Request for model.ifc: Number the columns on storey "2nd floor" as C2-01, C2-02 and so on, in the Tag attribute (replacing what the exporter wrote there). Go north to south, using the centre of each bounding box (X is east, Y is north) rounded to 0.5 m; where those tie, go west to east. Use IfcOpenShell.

First a look at what the model holds.

```python
import ifcopenshell
import ifcopenshell.util.element
import ifcopenshell.util.placement

model = ifcopenshell.open("model.ifc")
print(model.schema)
storey = next(s for s in model.by_type("IfcBuildingStorey") if s.Name == "2nd floor")
columns = [e for e in ifcopenshell.util.element.get_decomposition(storey) if e.is_a("IfcColumn")]
for e in sorted(columns, key=lambda e: e.id()):
    origin = ifcopenshell.util.placement.get_local_placement(e.ObjectPlacement)[:3, 3]
    print(e.id(), e.Tag, e.Name, origin.round(2) + 0.0, sep=" | ")
```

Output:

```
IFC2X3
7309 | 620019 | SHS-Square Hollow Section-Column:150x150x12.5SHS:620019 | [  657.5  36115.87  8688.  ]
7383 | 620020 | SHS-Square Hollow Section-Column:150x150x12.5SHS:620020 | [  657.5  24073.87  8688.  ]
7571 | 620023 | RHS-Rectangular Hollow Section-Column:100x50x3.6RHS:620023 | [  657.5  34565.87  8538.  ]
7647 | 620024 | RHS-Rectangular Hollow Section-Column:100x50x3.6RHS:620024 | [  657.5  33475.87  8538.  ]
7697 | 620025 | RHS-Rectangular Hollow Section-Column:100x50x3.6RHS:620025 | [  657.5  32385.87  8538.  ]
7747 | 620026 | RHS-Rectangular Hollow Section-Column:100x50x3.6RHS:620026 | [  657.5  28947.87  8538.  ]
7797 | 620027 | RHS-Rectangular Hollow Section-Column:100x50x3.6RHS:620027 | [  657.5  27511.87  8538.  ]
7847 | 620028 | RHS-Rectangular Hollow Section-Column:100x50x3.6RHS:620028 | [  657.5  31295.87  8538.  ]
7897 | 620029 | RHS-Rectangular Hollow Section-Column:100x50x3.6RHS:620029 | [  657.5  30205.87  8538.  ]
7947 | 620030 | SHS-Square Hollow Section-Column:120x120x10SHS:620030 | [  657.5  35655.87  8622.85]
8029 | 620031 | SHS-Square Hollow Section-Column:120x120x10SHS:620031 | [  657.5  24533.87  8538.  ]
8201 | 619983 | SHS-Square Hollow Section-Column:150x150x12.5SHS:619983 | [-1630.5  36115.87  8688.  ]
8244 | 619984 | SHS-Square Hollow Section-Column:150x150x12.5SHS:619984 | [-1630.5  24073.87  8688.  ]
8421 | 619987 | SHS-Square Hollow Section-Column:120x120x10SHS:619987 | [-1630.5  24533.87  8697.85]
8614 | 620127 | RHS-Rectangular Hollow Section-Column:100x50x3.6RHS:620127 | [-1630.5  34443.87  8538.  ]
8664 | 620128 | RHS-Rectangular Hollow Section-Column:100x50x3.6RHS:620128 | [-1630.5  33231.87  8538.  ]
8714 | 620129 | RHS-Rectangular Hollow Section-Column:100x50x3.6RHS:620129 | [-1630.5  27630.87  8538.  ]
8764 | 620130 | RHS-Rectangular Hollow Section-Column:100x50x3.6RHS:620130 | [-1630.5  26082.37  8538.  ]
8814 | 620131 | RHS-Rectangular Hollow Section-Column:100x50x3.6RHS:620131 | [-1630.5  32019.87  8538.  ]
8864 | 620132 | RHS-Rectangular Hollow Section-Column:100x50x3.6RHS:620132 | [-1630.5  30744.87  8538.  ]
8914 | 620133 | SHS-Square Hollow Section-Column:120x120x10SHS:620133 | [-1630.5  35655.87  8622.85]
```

```python
import ifcopenshell
import ifcopenshell.geom
import ifcopenshell.util.element
import ifcopenshell.util.shape

model = ifcopenshell.open("model.ifc")
settings = ifcopenshell.geom.settings()
settings.set("use-world-coords", True)


def centre(element):
    shape = ifcopenshell.geom.create_shape(settings, element)
    return ifcopenshell.util.shape.get_bbox_centroid(shape.geometry)


storey = next(s for s in model.by_type("IfcBuildingStorey") if s.Name == "2nd floor")
columns = [e for e in ifcopenshell.util.element.get_decomposition(storey) if e.is_a("IfcColumn")]

# Insertion points can sit at a corner or the storey origin, so sort by the geometry (in metres).
centres = {e: centre(e) for e in columns}
columns.sort(key=lambda e: (-round(centres[e][1] / 0.5), centres[e][0]))

for i, e in enumerate(columns, start=1):
    number = f"C2-{i:02d}"
    e.Tag = number
    print(e.id(), number)

model.write("model-out.ifc")
```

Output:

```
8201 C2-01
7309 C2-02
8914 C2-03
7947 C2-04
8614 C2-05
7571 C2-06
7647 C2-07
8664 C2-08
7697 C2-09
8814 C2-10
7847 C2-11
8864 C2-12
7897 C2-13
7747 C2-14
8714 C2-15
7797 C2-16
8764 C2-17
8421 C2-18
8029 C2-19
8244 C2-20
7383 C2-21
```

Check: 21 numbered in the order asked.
